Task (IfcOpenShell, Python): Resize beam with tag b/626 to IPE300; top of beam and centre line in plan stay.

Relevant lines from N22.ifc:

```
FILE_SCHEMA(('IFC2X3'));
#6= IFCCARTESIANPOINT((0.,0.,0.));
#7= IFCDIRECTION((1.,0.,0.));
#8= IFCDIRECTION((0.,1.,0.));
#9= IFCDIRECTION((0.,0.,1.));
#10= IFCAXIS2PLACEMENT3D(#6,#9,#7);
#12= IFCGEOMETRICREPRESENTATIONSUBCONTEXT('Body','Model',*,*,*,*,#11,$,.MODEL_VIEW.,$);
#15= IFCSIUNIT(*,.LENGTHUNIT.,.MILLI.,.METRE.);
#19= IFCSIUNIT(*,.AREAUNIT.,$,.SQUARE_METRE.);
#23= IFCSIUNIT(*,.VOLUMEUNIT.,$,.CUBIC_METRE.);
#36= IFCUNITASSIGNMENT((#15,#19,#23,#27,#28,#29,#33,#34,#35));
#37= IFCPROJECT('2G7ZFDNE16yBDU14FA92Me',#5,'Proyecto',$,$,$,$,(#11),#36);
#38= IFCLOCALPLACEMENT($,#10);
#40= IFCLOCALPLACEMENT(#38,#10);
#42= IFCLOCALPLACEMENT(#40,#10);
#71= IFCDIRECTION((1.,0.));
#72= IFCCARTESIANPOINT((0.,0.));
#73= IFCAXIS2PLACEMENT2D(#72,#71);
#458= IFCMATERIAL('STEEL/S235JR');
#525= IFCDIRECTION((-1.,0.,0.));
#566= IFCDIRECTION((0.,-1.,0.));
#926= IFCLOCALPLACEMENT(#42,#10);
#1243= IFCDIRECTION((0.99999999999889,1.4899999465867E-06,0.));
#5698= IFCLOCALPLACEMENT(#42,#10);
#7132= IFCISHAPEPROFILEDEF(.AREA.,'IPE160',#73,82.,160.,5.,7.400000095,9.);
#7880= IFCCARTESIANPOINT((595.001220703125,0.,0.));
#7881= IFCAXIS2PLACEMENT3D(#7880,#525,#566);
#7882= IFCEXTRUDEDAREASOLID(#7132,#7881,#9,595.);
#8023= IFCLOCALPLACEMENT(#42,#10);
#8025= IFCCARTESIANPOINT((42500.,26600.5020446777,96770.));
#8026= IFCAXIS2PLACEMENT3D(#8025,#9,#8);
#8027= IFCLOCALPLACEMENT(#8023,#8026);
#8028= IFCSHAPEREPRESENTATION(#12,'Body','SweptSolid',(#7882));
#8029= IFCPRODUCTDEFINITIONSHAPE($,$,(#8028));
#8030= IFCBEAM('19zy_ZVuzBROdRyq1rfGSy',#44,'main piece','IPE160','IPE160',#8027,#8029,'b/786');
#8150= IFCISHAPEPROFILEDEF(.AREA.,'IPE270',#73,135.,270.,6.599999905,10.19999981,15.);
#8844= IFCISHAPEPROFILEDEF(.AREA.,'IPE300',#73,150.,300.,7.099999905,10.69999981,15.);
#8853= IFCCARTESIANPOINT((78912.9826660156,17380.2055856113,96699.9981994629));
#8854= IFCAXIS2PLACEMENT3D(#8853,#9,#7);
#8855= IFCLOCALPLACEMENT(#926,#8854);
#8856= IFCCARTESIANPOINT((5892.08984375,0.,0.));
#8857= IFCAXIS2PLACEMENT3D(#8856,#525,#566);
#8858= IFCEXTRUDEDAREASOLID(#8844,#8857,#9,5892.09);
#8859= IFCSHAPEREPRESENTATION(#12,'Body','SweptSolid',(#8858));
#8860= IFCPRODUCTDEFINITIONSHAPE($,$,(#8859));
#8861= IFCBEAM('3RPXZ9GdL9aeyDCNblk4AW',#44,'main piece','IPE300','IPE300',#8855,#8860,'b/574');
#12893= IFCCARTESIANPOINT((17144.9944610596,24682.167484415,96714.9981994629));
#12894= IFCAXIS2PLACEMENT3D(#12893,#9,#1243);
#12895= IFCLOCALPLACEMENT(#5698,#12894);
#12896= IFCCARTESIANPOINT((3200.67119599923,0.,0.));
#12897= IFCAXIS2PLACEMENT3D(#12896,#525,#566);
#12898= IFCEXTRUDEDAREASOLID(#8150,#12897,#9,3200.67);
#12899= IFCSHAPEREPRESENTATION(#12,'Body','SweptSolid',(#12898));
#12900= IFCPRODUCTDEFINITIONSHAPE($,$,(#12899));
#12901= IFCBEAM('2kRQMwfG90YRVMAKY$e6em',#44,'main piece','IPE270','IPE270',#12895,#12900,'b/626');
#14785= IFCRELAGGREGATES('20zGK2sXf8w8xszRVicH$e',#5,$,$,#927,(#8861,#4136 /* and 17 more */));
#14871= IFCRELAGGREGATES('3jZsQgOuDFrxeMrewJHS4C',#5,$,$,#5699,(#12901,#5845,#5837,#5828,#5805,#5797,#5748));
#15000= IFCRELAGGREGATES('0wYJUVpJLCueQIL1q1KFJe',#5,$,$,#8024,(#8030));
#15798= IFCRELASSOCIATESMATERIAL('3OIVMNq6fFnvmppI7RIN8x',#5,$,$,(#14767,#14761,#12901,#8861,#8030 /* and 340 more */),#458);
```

```python
import ifcopenshell
import ifcopenshell.util.element
import ifcopenshell.util.representation

model = ifcopenshell.open("N22.ifc")

member = model.by_guid("2kRQMwfG90YRVMAKY$e6em")
source = next(p for p in model.by_type("IfcIShapeProfileDef") if p.ProfileName == "IPE300")

body = ifcopenshell.util.representation.get_representation(member, "Model", "Body")
solid = body.Items[0]
old_profile = solid.SweptArea

# Copy the section's sizes but keep this member's own profile position.
profile = ifcopenshell.util.element.copy(model, source)
# Profiles are centred, so shift by half the change in depth to hold the top.
shift = (old_profile.OverallDepth - profile.OverallDepth) / 2
x, y = old_profile.Position.Location.Coordinates
up = (0.0, 1.0)  # upwards, in the solid's own plane
location = model.createIfcCartesianPoint((x + up[0] * shift, y + up[1] * shift))
profile.Position = model.createIfcAxis2Placement2D(location, old_profile.Position.RefDirection)
solid.SweptArea = profile
if not model.get_total_inverses(old_profile):
    ifcopenshell.util.element.remove_deep2(model, old_profile)
member.Description = member.Description.replace("IPE270", "IPE300")
member.ObjectType = member.ObjectType.replace("IPE270", "IPE300")

print(solid.SweptArea)

model.write("N22_updated.ifc")
```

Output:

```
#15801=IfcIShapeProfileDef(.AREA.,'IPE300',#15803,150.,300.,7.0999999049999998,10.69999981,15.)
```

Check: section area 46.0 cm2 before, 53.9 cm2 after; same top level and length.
